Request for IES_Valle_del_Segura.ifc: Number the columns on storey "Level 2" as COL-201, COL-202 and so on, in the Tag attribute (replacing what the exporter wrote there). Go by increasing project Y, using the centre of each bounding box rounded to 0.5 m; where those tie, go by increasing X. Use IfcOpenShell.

First a look at what the model holds.

```python
import ifcopenshell
import ifcopenshell.util.element
import ifcopenshell.util.placement

model = ifcopenshell.open("IES_Valle_del_Segura.ifc")
print(model.schema)
storey = next(s for s in model.by_type("IfcBuildingStorey") if s.Name == "Level 2")
columns = [e for e in ifcopenshell.util.element.get_decomposition(storey) if e.is_a("IfcColumn")]
for e in sorted(columns, key=lambda e: e.id()):
    origin = ifcopenshell.util.placement.get_local_placement(e.ObjectPlacement)[:3, 3]
    print(e.id(), e.Tag, e.Name, origin.round(2) + 0.0, sep=" | ")
```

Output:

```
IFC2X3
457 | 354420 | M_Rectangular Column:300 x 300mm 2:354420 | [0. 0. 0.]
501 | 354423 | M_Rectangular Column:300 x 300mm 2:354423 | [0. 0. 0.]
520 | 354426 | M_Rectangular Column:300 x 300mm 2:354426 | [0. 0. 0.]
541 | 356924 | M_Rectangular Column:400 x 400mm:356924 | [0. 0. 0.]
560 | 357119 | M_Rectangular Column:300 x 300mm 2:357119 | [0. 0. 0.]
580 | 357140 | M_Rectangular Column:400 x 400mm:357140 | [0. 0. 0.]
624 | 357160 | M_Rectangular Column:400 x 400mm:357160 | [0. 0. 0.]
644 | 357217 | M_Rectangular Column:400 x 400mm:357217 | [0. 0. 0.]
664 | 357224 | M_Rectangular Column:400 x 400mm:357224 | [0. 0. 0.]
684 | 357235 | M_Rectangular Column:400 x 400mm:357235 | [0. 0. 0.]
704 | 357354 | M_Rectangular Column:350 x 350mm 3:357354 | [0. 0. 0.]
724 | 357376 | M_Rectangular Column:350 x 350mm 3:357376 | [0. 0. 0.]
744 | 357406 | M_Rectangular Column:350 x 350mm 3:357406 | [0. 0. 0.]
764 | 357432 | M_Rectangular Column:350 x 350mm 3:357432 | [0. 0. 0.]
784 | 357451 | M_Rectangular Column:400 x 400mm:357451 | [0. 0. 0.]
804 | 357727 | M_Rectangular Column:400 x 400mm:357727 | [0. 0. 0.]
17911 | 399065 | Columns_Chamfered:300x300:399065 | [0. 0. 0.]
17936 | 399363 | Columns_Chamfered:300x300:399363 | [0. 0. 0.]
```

```python
import ifcopenshell
import ifcopenshell.geom
import ifcopenshell.util.element
import ifcopenshell.util.shape

model = ifcopenshell.open("IES_Valle_del_Segura.ifc")
settings = ifcopenshell.geom.settings()
settings.set("use-world-coords", True)


def centre(element):
    shape = ifcopenshell.geom.create_shape(settings, element)
    return ifcopenshell.util.shape.get_bbox_centroid(shape.geometry)


storey = next(s for s in model.by_type("IfcBuildingStorey") if s.Name == "Level 2")
columns = [e for e in ifcopenshell.util.element.get_decomposition(storey) if e.is_a("IfcColumn")]

# Insertion points can sit at a corner or the storey origin, so sort by the geometry (in metres).
centres = {e: centre(e) for e in columns}
columns.sort(key=lambda e: (round(centres[e][1] / 0.5), centres[e][0]))

for i, e in enumerate(columns, start=1):
    number = f"COL-2{i:02d}"
    e.Tag = number
    print(e.id(), number)

model.write("IES_Valle_del_Segura-out.ifc")
```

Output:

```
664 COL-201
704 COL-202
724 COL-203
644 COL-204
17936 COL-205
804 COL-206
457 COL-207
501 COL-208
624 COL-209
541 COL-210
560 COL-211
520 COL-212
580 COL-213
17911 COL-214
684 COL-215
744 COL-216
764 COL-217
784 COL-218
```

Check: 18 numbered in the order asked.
